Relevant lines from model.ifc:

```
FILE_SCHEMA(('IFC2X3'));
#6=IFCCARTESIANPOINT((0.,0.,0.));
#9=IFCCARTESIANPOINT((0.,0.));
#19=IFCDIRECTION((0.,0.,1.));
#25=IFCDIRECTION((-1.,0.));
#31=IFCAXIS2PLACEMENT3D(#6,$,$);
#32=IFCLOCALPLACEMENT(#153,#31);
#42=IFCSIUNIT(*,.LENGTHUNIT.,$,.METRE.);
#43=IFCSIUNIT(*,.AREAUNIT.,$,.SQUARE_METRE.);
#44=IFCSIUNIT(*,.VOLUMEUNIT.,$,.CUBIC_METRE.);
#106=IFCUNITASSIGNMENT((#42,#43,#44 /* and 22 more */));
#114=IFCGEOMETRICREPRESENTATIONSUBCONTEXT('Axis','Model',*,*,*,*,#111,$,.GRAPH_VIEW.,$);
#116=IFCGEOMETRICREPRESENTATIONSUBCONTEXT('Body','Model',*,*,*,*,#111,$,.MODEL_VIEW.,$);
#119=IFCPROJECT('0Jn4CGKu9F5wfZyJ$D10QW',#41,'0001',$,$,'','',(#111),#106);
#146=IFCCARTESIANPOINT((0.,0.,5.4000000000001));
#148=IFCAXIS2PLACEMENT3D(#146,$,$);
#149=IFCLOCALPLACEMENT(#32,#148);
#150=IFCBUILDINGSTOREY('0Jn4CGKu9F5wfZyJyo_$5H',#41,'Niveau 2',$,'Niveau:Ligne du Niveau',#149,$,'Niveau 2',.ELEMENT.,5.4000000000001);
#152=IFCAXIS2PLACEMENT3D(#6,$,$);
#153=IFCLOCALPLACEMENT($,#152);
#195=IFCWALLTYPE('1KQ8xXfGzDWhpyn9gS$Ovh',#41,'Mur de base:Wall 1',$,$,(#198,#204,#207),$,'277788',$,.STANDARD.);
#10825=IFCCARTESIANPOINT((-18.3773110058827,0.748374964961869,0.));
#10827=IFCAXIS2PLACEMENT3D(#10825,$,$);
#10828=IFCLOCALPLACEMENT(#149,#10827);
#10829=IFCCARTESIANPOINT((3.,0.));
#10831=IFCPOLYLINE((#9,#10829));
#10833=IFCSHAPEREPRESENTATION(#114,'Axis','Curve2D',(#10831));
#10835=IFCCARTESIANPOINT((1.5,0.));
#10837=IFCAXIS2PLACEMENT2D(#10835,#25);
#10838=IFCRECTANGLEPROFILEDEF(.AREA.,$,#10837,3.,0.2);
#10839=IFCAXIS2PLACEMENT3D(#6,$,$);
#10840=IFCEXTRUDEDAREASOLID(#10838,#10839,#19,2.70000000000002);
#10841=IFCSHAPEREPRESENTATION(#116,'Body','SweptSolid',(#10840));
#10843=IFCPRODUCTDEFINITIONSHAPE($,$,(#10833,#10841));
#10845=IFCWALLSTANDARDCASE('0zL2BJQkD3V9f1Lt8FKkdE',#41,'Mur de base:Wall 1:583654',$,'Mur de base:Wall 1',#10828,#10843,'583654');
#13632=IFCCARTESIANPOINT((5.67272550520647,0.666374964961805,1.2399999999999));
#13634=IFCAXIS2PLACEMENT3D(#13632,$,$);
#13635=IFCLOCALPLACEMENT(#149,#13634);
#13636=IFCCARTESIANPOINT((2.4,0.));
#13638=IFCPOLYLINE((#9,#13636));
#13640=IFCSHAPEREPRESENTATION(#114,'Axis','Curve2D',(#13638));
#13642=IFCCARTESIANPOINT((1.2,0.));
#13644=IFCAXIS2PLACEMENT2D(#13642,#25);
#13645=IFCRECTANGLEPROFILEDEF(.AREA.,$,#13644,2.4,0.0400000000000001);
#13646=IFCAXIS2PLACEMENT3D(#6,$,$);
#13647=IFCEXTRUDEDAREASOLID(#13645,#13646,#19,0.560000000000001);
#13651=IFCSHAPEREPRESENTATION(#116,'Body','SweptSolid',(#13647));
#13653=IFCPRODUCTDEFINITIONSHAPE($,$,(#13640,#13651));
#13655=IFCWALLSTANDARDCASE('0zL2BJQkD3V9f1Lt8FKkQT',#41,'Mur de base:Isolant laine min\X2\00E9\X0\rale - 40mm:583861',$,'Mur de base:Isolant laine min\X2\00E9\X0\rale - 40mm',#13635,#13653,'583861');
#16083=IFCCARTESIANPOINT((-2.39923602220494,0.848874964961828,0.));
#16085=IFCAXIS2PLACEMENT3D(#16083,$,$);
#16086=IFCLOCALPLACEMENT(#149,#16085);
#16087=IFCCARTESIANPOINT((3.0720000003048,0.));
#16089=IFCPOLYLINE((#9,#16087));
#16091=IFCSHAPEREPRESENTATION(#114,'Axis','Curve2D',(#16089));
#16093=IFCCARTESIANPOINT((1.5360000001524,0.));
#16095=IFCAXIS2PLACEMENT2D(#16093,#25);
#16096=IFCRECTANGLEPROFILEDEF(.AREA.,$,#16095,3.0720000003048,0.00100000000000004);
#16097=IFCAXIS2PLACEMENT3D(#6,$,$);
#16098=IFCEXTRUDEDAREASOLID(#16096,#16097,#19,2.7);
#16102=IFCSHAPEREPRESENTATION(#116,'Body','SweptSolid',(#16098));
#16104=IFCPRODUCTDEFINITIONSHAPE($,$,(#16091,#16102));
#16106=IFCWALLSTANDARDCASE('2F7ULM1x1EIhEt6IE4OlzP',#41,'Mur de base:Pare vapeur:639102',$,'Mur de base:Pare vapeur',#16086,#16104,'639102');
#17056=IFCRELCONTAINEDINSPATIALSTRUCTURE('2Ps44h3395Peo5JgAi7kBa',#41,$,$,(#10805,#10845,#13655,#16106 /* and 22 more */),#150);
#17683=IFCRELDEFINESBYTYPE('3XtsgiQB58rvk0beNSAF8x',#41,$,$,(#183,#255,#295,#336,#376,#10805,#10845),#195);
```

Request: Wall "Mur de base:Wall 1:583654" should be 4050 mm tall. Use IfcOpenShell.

```python
import ifcopenshell
import ifcopenshell.geom
import ifcopenshell.util.representation
import ifcopenshell.util.shape
import ifcopenshell.util.unit

model = ifcopenshell.open("model.ifc")
unit_scale = ifcopenshell.util.unit.calculate_unit_scale(model)
settings = ifcopenshell.geom.settings()


def volume(element):
    """Net volume in cubic metres, openings subtracted."""
    shape = ifcopenshell.geom.create_shape(settings, element)
    return ifcopenshell.util.shape.get_volume(shape.geometry)


wall = model.by_id(10845)
before = volume(wall)

body = ifcopenshell.util.representation.get_representation(wall, "Model", "Body")
solid = body.Items[0]
old_height = solid.Depth
solid.Depth = 4.05 / unit_scale
after = volume(wall)

print(f"height {old_height:g} -> {solid.Depth:g}, volume {before:.3f} -> {after:.3f} m3")

model.write("model_v2.ifc")
```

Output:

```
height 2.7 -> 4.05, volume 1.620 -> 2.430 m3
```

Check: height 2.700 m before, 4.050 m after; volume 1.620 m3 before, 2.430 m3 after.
